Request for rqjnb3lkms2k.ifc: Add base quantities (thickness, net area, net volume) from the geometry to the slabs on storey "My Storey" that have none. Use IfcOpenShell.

First a look at what the model holds.

```python
import ifcopenshell
import ifcopenshell.util.element
import ifcopenshell.util.unit

model = ifcopenshell.open("rqjnb3lkms2k.ifc")
print(model.schema)
for unit_type in ("LENGTHUNIT", "AREAUNIT", "VOLUMEUNIT"):
    print(unit_type, ifcopenshell.util.unit.calculate_unit_scale(model, unit_type))
storey = next(s for s in model.by_type("IfcBuildingStorey") if s.Name == "My Storey")
slabs = [e for e in ifcopenshell.util.element.get_decomposition(storey) if e.is_a("IfcSlab")]
for e in sorted(slabs, key=lambda e: e.id()):
    print(e.id(), e.is_a(), e.Name, list(ifcopenshell.util.element.get_psets(e, qtos_only=True)), sep=" | ")
```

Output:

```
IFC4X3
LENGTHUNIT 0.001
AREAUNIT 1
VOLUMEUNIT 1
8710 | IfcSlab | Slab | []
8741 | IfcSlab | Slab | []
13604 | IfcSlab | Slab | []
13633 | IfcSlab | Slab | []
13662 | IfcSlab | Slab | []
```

```python
import ifcopenshell
import ifcopenshell.api.pset
import ifcopenshell.geom
import ifcopenshell.util.element
import ifcopenshell.util.shape
import ifcopenshell.util.unit

model = ifcopenshell.open("rqjnb3lkms2k.ifc")
unit_scale = ifcopenshell.util.unit.calculate_unit_scale(model)
area_scale = ifcopenshell.util.unit.calculate_unit_scale(model, "AREAUNIT")
volume_scale = ifcopenshell.util.unit.calculate_unit_scale(model, "VOLUMEUNIT")
settings = ifcopenshell.geom.settings()

storey = next(s for s in model.by_type("IfcBuildingStorey") if s.Name == "My Storey")
slabs = [e for e in ifcopenshell.util.element.get_decomposition(storey) if e.is_a("IfcSlab")]

for e in sorted(slabs, key=lambda e: e.id()):
    if ifcopenshell.util.element.get_psets(e, qtos_only=True, should_inherit=False):
        continue
    # Geometry comes back in metres, in the element's own axes.
    shape = ifcopenshell.geom.create_shape(settings, e)
    values = {
        "Width": ifcopenshell.util.shape.get_z(shape.geometry) / unit_scale,
        "NetArea": ifcopenshell.util.shape.get_footprint_area(shape.geometry) / area_scale,
        "NetVolume": ifcopenshell.util.shape.get_volume(shape.geometry) / volume_scale,
    }
    qto = ifcopenshell.api.pset.add_qto(model, product=e, name="Qto_SlabBaseQuantities")
    ifcopenshell.api.pset.edit_qto(model, qto=qto, properties=values)
    print(e.id(), {k: round(v, 3) for k, v in values.items()})

model.write("rqjnb3lkms2k_updated.ifc")
```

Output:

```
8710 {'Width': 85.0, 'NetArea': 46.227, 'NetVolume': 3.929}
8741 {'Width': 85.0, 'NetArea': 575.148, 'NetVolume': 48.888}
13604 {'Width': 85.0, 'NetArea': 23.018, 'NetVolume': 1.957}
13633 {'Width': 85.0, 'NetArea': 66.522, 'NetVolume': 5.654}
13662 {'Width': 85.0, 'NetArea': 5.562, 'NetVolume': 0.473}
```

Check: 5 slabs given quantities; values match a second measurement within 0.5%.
